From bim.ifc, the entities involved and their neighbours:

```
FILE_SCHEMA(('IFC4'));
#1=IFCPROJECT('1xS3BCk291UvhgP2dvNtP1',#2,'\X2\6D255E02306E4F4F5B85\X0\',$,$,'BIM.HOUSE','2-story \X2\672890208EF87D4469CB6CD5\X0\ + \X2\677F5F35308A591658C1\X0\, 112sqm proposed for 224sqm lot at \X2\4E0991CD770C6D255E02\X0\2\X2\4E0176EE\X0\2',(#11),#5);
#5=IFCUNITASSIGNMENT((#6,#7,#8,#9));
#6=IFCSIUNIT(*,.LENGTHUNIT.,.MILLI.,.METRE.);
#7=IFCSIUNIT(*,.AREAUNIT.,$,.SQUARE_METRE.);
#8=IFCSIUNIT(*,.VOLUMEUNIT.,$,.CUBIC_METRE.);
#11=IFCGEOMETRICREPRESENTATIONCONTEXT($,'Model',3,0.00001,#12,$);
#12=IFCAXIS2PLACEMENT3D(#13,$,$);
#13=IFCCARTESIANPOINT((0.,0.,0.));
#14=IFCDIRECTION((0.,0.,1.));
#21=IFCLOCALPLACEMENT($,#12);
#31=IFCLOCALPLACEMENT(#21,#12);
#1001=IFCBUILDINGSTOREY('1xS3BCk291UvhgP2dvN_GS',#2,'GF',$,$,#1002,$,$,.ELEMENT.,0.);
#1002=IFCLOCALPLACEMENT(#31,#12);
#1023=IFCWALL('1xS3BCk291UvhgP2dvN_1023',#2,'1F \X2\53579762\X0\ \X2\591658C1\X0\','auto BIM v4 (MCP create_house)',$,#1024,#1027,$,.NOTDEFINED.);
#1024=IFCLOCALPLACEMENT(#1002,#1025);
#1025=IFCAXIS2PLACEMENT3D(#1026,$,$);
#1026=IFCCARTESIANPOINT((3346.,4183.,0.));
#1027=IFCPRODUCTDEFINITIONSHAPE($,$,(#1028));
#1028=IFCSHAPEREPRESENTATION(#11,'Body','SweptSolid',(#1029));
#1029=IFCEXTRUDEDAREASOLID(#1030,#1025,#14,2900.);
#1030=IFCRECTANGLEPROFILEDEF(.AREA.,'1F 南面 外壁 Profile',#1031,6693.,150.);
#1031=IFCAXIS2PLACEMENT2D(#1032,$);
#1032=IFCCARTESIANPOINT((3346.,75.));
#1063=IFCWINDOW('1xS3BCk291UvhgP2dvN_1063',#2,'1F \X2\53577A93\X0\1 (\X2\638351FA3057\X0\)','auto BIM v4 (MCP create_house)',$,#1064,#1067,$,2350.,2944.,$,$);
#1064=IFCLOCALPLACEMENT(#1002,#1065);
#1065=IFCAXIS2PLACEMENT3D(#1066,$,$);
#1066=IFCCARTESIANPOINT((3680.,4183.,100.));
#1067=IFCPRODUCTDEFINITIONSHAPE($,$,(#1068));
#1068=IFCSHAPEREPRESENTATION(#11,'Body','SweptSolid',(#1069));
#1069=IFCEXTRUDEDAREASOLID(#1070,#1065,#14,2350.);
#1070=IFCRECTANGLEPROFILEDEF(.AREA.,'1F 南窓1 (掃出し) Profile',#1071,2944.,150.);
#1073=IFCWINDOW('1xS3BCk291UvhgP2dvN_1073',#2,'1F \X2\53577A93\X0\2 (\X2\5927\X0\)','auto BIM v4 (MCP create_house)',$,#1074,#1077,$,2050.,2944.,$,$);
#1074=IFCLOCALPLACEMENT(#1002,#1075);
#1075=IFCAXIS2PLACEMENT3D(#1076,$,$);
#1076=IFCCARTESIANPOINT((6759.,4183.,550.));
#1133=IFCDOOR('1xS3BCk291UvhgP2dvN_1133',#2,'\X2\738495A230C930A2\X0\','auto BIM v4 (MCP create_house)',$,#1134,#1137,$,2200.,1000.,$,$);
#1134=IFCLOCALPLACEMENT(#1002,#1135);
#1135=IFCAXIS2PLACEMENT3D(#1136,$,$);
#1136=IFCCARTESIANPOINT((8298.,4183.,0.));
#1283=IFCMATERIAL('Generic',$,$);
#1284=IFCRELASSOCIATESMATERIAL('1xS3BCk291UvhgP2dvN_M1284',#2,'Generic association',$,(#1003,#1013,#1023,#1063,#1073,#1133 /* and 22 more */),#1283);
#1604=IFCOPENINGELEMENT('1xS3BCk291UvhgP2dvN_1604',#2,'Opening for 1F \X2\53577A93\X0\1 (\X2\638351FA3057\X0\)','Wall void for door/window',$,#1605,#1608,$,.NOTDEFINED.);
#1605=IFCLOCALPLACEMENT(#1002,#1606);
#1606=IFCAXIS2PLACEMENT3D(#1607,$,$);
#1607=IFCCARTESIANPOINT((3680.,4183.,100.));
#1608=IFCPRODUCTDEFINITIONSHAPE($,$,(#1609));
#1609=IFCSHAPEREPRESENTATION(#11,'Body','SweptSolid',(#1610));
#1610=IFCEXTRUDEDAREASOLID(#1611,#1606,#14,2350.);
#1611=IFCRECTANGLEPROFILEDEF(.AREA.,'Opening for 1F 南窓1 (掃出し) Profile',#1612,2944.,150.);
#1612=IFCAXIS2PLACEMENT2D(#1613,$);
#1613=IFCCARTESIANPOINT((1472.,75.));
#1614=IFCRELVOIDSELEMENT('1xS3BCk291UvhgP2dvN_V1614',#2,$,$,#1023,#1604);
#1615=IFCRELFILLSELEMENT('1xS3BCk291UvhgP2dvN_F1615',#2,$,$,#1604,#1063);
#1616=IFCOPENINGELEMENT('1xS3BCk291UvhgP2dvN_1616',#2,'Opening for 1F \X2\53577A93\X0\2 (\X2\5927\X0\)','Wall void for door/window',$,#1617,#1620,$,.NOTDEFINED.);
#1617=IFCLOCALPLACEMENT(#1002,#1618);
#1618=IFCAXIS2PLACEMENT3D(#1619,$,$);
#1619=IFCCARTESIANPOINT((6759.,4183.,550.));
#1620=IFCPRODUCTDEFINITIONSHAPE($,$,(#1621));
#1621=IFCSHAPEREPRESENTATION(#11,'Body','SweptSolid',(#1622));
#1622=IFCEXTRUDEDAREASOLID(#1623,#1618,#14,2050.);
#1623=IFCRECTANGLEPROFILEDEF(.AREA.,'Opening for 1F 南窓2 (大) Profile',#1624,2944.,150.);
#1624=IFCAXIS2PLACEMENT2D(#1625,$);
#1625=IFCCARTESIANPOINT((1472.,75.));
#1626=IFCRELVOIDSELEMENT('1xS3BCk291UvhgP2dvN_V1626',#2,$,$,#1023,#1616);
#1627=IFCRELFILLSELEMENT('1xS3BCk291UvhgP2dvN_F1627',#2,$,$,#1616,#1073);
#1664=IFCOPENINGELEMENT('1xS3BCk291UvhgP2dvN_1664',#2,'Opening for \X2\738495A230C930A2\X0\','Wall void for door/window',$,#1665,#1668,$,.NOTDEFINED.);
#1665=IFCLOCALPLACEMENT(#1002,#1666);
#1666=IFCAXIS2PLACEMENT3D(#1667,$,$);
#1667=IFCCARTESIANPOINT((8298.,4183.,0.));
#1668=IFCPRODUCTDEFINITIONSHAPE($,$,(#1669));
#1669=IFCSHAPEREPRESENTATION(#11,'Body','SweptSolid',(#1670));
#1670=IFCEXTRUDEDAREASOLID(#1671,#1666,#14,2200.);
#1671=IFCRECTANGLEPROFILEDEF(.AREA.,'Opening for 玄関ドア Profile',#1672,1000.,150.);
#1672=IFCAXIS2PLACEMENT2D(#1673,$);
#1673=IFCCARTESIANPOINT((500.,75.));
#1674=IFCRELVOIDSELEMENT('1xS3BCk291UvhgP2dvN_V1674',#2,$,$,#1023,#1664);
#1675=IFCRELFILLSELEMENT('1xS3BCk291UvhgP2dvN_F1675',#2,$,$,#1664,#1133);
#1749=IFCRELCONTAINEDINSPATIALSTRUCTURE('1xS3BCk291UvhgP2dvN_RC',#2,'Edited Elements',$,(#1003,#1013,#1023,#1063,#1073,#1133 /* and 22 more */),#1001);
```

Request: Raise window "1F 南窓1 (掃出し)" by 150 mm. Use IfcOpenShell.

```python
import numpy as np
import ifcopenshell
import ifcopenshell.api.geometry
import ifcopenshell.util.placement
import ifcopenshell.util.unit

model = ifcopenshell.open("bim.ifc")
unit_scale = ifcopenshell.util.unit.calculate_unit_scale(model)

window = model.by_id(1063)
opening = window.FillsVoids[0].RelatingOpeningElement
dz = 150.0

shift = np.array([0.0, 0.0, dz])
# The window is not placed relative to its opening, so move both.
for product in (opening, window):
    matrix = ifcopenshell.util.placement.get_local_placement(product.ObjectPlacement)
    matrix[:3, 3] += shift
    ifcopenshell.api.geometry.edit_object_placement(model, product=product, matrix=matrix, is_si=False)

print(f"moved by {dz * unit_scale:+.3f} m")

model.write("bim_v2.ifc")
```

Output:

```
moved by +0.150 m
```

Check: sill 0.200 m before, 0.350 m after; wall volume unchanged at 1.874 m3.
